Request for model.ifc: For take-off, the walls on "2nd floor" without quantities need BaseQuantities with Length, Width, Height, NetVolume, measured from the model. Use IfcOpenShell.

First a look at what the model holds.

```python
import ifcopenshell
import ifcopenshell.util.element
import ifcopenshell.util.unit

model = ifcopenshell.open("model.ifc")
print(model.schema)
for unit_type in ("LENGTHUNIT", "AREAUNIT", "VOLUMEUNIT"):
    print(unit_type, ifcopenshell.util.unit.calculate_unit_scale(model, unit_type))
storey = next(s for s in model.by_type("IfcBuildingStorey") if s.Name == "2nd floor")
walls = [e for e in ifcopenshell.util.element.get_decomposition(storey) if e.is_a("IfcWall")]
for e in sorted(walls, key=lambda e: e.id()):
    print(e.id(), e.is_a(), e.Name, list(ifcopenshell.util.element.get_psets(e, qtos_only=True)), sep=" | ")
```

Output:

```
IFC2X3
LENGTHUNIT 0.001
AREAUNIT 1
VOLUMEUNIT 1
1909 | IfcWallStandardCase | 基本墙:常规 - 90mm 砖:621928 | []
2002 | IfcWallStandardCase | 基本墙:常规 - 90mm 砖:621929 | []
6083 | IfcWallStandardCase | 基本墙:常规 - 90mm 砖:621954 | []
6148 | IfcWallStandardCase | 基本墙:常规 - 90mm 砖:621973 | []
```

```python
import ifcopenshell
import ifcopenshell.api.pset
import ifcopenshell.geom
import ifcopenshell.util.element
import ifcopenshell.util.shape
import ifcopenshell.util.unit

model = ifcopenshell.open("model.ifc")
unit_scale = ifcopenshell.util.unit.calculate_unit_scale(model)
volume_scale = ifcopenshell.util.unit.calculate_unit_scale(model, "VOLUMEUNIT")
settings = ifcopenshell.geom.settings()

storey = next(s for s in model.by_type("IfcBuildingStorey") if s.Name == "2nd floor")
walls = [e for e in ifcopenshell.util.element.get_decomposition(storey) if e.is_a("IfcWall")]

for e in sorted(walls, key=lambda e: e.id()):
    if ifcopenshell.util.element.get_psets(e, qtos_only=True, should_inherit=False):
        continue
    # Geometry comes back in metres, in the element's own axes.
    shape = ifcopenshell.geom.create_shape(settings, e)
    values = {
        "Length": ifcopenshell.util.shape.get_x(shape.geometry) / unit_scale,
        "Width": ifcopenshell.util.shape.get_y(shape.geometry) / unit_scale,
        "Height": ifcopenshell.util.shape.get_z(shape.geometry) / unit_scale,
        "NetVolume": ifcopenshell.util.shape.get_volume(shape.geometry) / volume_scale,
    }
    qto = ifcopenshell.api.pset.add_qto(model, product=e, name="BaseQuantities")
    ifcopenshell.api.pset.edit_qto(model, qto=qto, properties=values)
    print(e.id(), {k: round(v, 3) for k, v in values.items()})

model.write("model_v2.ifc")
```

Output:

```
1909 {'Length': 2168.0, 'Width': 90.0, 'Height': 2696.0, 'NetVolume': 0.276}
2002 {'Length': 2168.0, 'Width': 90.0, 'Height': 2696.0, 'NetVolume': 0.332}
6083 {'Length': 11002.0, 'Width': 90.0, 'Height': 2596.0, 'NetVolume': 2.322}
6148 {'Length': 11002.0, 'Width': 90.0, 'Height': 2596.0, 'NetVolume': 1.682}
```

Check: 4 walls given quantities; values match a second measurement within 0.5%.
